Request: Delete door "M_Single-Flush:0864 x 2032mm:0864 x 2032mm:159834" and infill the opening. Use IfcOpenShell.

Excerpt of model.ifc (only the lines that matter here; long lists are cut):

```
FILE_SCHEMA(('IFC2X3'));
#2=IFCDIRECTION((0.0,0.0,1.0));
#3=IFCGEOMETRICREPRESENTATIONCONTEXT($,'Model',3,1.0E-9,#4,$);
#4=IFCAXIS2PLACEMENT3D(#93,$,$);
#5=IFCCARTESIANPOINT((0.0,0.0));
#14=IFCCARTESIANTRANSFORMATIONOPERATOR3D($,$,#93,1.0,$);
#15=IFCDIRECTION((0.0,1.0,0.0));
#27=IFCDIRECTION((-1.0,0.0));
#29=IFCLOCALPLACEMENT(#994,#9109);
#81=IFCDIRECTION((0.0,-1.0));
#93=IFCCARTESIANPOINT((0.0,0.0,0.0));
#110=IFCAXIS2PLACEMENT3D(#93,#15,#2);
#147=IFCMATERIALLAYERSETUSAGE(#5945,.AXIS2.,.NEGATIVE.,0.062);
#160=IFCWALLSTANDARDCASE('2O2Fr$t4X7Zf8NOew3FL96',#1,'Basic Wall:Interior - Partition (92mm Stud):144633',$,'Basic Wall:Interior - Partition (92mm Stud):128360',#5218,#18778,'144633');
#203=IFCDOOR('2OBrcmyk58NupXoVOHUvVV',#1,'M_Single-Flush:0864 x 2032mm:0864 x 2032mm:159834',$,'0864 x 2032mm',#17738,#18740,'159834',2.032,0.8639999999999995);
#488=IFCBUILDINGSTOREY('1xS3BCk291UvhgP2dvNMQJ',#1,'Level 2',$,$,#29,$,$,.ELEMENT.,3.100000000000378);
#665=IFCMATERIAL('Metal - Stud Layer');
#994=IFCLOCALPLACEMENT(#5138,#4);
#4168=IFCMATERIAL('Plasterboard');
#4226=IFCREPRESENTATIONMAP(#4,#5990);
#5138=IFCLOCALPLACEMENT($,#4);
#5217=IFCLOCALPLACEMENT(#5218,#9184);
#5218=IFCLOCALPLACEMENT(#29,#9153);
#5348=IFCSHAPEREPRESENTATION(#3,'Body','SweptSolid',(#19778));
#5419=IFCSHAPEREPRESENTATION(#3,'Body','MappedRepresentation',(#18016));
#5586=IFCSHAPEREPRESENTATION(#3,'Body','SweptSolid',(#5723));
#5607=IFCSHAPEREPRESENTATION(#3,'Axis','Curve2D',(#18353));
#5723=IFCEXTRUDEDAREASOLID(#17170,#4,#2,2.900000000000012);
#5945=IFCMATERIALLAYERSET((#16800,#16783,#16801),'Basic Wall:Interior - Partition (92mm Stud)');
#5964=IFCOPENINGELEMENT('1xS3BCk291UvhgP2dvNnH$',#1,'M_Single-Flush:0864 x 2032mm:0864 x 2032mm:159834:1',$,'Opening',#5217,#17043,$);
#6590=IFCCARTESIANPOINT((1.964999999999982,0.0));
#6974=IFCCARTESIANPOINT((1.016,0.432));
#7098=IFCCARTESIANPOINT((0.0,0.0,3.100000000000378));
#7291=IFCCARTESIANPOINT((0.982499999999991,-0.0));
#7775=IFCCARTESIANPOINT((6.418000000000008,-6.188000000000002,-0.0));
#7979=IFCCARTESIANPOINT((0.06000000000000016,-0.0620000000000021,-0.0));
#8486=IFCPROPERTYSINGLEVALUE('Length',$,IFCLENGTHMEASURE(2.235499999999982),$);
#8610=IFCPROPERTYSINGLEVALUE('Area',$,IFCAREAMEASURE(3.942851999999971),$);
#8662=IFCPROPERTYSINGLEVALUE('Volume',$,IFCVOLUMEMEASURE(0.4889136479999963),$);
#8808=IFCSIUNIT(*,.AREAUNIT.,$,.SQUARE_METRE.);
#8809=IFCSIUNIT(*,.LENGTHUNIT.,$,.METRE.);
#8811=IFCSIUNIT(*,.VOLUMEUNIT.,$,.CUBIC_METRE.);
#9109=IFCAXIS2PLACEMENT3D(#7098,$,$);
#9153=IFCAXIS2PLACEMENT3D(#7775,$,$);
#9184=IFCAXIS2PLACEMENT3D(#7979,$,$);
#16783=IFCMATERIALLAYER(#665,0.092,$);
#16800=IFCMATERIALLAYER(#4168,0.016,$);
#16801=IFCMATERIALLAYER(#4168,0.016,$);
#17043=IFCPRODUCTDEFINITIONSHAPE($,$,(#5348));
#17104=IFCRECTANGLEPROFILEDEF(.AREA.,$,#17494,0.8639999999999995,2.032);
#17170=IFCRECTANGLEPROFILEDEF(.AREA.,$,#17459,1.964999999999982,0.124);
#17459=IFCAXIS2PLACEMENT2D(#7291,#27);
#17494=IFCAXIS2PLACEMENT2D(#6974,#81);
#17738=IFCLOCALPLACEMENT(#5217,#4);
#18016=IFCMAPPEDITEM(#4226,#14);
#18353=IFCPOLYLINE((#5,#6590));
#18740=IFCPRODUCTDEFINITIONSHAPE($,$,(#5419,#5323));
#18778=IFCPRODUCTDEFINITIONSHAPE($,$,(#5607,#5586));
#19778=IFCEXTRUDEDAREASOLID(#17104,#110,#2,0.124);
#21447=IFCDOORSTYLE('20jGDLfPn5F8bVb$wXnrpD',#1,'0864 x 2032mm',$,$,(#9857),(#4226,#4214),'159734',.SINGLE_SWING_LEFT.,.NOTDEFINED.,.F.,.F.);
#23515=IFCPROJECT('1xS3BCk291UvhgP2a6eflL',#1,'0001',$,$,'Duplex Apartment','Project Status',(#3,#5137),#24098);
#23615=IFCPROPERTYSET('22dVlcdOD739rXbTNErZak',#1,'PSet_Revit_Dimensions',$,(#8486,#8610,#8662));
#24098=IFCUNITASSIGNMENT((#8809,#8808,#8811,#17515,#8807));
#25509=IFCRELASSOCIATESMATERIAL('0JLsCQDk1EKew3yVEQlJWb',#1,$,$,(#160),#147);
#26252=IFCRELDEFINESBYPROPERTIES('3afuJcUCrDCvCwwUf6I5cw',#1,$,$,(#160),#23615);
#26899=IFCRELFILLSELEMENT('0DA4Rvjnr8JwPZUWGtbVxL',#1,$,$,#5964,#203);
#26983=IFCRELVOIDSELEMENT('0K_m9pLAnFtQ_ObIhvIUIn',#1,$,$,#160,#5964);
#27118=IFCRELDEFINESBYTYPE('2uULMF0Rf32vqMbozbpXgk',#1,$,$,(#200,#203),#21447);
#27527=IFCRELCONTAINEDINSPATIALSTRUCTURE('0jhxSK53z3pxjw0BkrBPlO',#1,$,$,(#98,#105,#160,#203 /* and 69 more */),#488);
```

```python
import ifcopenshell
import ifcopenshell.api.feature
import ifcopenshell.api.pset
import ifcopenshell.api.root
import ifcopenshell.geom
import ifcopenshell.util.element
import ifcopenshell.util.shape
import ifcopenshell.util.unit

model = ifcopenshell.open("model.ifc")
area_scale = ifcopenshell.util.unit.calculate_unit_scale(model, "AREAUNIT")
volume_scale = ifcopenshell.util.unit.calculate_unit_scale(model, "VOLUMEUNIT")
settings = ifcopenshell.geom.settings()


def volume(element):
    """Net volume in cubic metres, openings subtracted."""
    shape = ifcopenshell.geom.create_shape(settings, element)
    return ifcopenshell.util.shape.get_volume(shape.geometry)


door = model.by_id(203)
opening = door.FillsVoids[0].RelatingOpeningElement
wall = opening.VoidsElements[0].RelatingBuildingElement
before = volume(wall)

ifcopenshell.api.root.remove_product(model, product=door)
ifcopenshell.api.feature.remove_feature(model, feature=opening)

after = volume(wall)
thickness = 0.124  # wall thickness in metres

# Update the wall's stored quantities.
pset = model.by_id(ifcopenshell.util.element.get_pset(wall, "PSet_Revit_Dimensions", should_inherit=False)["id"])
ifcopenshell.api.pset.edit_pset(model, pset=pset, properties={
    "Area": model.create_entity("IfcAreaMeasure", after / thickness / area_scale),
    "Volume": model.create_entity("IfcVolumeMeasure", after / volume_scale),
})

print(f"wall volume {before:.3f} -> {after:.3f} m3")

model.write("model_updated.ifc")
```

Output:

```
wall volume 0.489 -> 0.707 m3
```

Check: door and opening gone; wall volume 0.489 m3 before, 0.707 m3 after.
